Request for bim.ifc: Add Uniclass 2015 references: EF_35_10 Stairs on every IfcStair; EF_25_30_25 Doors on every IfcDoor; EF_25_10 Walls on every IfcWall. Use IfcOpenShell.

First a look at what the model holds.

```python
import ifcopenshell

model = ifcopenshell.open("bim.ifc")
print(model.schema)
print("classifications:", [c.Name for c in model.by_type("IfcClassification")])
for ifc_class in ("IfcDoor", "IfcRoof", "IfcStair", "IfcWall", "IfcWindow"):
    print(ifc_class, len(model.by_type(ifc_class)))
```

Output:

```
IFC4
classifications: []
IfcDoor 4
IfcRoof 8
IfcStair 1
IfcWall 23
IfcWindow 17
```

```python
import ifcopenshell
import ifcopenshell.api.classification

model = ifcopenshell.open("bim.ifc")

system = ifcopenshell.api.classification.add_classification(model, classification="Uniclass 2015")

codes = {
    "IfcStair": ("EF_35_10", "Stairs"),
    "IfcDoor": ("EF_25_30_25", "Doors"),
    "IfcWall": ("EF_25_10", "Walls"),
}
for ifc_class, (code, name) in codes.items():
    products = model.by_type(ifc_class)
    ifcopenshell.api.classification.add_reference(
        model, products=products, classification=system, identification=code, name=name
    )
    print(code, len(products))

model.write("bim_rev.ifc")
```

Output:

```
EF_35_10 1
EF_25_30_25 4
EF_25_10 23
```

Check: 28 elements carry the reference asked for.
